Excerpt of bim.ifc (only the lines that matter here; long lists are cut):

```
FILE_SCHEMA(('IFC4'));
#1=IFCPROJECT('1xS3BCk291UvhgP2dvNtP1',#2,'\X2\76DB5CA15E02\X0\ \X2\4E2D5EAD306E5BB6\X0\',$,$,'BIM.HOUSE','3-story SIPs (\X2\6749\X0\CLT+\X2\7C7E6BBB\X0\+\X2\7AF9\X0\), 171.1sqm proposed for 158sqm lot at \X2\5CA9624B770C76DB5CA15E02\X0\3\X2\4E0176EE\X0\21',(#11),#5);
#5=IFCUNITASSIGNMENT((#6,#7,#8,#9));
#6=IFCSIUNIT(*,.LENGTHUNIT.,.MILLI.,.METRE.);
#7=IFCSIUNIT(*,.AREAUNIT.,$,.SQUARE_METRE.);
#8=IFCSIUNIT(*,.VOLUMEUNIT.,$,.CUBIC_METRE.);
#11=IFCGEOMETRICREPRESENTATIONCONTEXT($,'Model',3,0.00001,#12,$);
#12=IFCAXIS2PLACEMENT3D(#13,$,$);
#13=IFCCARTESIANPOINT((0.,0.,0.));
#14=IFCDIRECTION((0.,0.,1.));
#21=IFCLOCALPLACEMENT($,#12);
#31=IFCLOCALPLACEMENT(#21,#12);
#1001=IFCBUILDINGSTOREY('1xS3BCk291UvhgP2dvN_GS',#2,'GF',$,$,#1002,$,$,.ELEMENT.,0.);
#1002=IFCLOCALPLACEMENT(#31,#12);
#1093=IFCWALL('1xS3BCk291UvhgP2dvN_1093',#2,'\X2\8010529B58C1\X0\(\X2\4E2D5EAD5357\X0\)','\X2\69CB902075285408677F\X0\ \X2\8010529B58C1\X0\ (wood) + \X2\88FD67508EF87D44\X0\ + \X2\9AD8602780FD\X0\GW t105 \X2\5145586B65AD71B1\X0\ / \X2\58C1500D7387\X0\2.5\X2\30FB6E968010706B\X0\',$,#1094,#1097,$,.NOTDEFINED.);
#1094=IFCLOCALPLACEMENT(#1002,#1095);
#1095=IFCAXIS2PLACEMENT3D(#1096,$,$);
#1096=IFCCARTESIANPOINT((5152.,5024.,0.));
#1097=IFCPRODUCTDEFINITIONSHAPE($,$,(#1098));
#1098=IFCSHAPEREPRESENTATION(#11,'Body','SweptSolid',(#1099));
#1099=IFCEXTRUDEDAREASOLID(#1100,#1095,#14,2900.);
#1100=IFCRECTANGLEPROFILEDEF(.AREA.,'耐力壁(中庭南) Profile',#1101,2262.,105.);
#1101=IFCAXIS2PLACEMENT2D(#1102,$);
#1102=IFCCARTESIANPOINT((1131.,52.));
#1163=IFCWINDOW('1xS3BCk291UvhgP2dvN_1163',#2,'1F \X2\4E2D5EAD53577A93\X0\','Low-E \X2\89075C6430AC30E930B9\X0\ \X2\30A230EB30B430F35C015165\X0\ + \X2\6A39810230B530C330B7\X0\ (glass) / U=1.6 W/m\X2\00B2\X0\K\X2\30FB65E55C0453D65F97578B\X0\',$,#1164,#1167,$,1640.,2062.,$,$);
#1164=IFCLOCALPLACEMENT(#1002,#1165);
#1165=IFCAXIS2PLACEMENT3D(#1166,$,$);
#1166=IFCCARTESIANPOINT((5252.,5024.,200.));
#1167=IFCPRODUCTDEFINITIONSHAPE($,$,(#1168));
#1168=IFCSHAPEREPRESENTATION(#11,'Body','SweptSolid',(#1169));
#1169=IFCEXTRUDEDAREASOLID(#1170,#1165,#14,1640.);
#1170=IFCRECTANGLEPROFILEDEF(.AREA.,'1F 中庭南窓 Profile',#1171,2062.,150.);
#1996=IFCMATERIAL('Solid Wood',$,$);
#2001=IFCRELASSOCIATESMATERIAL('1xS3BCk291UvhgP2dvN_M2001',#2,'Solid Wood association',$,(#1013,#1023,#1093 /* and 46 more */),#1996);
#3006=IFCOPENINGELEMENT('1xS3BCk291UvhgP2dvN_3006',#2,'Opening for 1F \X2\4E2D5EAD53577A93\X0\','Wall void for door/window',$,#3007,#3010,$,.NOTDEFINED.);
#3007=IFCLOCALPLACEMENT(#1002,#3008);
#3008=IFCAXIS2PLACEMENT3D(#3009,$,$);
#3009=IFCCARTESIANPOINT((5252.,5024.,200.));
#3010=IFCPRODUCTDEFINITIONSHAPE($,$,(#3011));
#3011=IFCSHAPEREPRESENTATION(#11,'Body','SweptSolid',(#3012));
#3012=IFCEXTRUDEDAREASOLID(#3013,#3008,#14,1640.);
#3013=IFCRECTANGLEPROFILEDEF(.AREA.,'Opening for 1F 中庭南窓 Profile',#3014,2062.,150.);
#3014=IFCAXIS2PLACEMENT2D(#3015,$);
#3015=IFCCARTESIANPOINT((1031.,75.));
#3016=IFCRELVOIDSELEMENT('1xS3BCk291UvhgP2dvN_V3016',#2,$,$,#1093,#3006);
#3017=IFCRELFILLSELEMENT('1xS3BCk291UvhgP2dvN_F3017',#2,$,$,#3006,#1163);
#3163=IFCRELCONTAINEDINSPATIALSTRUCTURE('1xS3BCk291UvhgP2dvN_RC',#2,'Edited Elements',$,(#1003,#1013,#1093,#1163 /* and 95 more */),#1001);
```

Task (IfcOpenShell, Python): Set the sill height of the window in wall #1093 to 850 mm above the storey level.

```python
import numpy as np
import ifcopenshell
import ifcopenshell.api.geometry
import ifcopenshell.geom
import ifcopenshell.util.element
import ifcopenshell.util.placement
import ifcopenshell.util.shape
import ifcopenshell.util.unit

model = ifcopenshell.open("bim.ifc")
unit_scale = ifcopenshell.util.unit.calculate_unit_scale(model)

window = model.by_guid("1xS3BCk291UvhgP2dvN_1163")
opening = window.FillsVoids[0].RelatingOpeningElement
storey = ifcopenshell.util.element.get_container(window, ifc_class="IfcBuildingStorey")
level = ifcopenshell.util.placement.get_local_placement(storey.ObjectPlacement)[2, 3]

# The opening's origin need not be at the sill, so measure its lowest point.
shape = ifcopenshell.geom.create_shape(ifcopenshell.geom.settings(), opening)
bottom = ifcopenshell.util.shape.get_shape_bottom_elevation(shape, shape.geometry) / unit_scale
dz = level + 0.85 / unit_scale - bottom

shift = np.array([0.0, 0.0, dz])
# The window is not placed relative to its opening, so move both.
for product in (opening, window):
    matrix = ifcopenshell.util.placement.get_local_placement(product.ObjectPlacement)
    matrix[:3, 3] += shift
    ifcopenshell.api.geometry.edit_object_placement(model, product=product, matrix=matrix, is_si=False)

print(f"moved by {dz * unit_scale:+.3f} m")

model.write("bim_v2.ifc")
```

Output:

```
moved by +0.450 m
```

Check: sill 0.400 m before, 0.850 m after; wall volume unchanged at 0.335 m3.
